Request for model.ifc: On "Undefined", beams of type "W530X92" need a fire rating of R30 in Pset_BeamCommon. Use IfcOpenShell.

First a look at what the model holds.

```python
import ifcopenshell
import ifcopenshell.util.element

model = ifcopenshell.open("model.ifc")
print(model.schema)
storey = next(s for s in model.by_type("IfcBuildingStorey") if s.Name == "Undefined")
beams = [e for e in ifcopenshell.util.element.get_decomposition(storey) if e.is_a("IfcBeam")]
seen = {}
for e in beams:
    element_type = ifcopenshell.util.element.get_type(e)
    key = (element_type.Name if element_type != e and element_type else None, ifcopenshell.util.element.get_pset(e, "Pset_BeamCommon", "FireRating"))
    seen[key] = seen.get(key, 0) + 1
for (name, value), count in sorted(seen.items(), key=str):
    print(count, "x", name, "|", value)
```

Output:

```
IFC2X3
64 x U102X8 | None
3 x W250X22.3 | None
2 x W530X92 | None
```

```python
import ifcopenshell
import ifcopenshell.api.pset
import ifcopenshell.util.element

model = ifcopenshell.open("model.ifc")

storey = next(s for s in model.by_type("IfcBuildingStorey") if s.Name == "Undefined")
beams = [e for e in ifcopenshell.util.element.get_decomposition(storey) if e.is_a("IfcBeam")]

count = 0
for e in beams:
    element_type = ifcopenshell.util.element.get_type(e)
    if element_type in (None, e) or element_type.Name != "W530X92":
        continue
    found = ifcopenshell.util.element.get_pset(e, "Pset_BeamCommon", should_inherit=False)
    if found:
        pset = model.by_id(found["id"])
        if len(ifcopenshell.util.element.get_elements_by_pset(pset)) > 1:
            pset = ifcopenshell.api.pset.unshare_pset(model, products=[e], pset=pset)[0]
    else:
        pset = ifcopenshell.api.pset.add_pset(model, product=e, name="Pset_BeamCommon")
    ifcopenshell.api.pset.edit_pset(model, pset=pset, properties={"FireRating": "R30"})
    count += 1

print(count, "beams updated")

model.write("model_updated.ifc")
```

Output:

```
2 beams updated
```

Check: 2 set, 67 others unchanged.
